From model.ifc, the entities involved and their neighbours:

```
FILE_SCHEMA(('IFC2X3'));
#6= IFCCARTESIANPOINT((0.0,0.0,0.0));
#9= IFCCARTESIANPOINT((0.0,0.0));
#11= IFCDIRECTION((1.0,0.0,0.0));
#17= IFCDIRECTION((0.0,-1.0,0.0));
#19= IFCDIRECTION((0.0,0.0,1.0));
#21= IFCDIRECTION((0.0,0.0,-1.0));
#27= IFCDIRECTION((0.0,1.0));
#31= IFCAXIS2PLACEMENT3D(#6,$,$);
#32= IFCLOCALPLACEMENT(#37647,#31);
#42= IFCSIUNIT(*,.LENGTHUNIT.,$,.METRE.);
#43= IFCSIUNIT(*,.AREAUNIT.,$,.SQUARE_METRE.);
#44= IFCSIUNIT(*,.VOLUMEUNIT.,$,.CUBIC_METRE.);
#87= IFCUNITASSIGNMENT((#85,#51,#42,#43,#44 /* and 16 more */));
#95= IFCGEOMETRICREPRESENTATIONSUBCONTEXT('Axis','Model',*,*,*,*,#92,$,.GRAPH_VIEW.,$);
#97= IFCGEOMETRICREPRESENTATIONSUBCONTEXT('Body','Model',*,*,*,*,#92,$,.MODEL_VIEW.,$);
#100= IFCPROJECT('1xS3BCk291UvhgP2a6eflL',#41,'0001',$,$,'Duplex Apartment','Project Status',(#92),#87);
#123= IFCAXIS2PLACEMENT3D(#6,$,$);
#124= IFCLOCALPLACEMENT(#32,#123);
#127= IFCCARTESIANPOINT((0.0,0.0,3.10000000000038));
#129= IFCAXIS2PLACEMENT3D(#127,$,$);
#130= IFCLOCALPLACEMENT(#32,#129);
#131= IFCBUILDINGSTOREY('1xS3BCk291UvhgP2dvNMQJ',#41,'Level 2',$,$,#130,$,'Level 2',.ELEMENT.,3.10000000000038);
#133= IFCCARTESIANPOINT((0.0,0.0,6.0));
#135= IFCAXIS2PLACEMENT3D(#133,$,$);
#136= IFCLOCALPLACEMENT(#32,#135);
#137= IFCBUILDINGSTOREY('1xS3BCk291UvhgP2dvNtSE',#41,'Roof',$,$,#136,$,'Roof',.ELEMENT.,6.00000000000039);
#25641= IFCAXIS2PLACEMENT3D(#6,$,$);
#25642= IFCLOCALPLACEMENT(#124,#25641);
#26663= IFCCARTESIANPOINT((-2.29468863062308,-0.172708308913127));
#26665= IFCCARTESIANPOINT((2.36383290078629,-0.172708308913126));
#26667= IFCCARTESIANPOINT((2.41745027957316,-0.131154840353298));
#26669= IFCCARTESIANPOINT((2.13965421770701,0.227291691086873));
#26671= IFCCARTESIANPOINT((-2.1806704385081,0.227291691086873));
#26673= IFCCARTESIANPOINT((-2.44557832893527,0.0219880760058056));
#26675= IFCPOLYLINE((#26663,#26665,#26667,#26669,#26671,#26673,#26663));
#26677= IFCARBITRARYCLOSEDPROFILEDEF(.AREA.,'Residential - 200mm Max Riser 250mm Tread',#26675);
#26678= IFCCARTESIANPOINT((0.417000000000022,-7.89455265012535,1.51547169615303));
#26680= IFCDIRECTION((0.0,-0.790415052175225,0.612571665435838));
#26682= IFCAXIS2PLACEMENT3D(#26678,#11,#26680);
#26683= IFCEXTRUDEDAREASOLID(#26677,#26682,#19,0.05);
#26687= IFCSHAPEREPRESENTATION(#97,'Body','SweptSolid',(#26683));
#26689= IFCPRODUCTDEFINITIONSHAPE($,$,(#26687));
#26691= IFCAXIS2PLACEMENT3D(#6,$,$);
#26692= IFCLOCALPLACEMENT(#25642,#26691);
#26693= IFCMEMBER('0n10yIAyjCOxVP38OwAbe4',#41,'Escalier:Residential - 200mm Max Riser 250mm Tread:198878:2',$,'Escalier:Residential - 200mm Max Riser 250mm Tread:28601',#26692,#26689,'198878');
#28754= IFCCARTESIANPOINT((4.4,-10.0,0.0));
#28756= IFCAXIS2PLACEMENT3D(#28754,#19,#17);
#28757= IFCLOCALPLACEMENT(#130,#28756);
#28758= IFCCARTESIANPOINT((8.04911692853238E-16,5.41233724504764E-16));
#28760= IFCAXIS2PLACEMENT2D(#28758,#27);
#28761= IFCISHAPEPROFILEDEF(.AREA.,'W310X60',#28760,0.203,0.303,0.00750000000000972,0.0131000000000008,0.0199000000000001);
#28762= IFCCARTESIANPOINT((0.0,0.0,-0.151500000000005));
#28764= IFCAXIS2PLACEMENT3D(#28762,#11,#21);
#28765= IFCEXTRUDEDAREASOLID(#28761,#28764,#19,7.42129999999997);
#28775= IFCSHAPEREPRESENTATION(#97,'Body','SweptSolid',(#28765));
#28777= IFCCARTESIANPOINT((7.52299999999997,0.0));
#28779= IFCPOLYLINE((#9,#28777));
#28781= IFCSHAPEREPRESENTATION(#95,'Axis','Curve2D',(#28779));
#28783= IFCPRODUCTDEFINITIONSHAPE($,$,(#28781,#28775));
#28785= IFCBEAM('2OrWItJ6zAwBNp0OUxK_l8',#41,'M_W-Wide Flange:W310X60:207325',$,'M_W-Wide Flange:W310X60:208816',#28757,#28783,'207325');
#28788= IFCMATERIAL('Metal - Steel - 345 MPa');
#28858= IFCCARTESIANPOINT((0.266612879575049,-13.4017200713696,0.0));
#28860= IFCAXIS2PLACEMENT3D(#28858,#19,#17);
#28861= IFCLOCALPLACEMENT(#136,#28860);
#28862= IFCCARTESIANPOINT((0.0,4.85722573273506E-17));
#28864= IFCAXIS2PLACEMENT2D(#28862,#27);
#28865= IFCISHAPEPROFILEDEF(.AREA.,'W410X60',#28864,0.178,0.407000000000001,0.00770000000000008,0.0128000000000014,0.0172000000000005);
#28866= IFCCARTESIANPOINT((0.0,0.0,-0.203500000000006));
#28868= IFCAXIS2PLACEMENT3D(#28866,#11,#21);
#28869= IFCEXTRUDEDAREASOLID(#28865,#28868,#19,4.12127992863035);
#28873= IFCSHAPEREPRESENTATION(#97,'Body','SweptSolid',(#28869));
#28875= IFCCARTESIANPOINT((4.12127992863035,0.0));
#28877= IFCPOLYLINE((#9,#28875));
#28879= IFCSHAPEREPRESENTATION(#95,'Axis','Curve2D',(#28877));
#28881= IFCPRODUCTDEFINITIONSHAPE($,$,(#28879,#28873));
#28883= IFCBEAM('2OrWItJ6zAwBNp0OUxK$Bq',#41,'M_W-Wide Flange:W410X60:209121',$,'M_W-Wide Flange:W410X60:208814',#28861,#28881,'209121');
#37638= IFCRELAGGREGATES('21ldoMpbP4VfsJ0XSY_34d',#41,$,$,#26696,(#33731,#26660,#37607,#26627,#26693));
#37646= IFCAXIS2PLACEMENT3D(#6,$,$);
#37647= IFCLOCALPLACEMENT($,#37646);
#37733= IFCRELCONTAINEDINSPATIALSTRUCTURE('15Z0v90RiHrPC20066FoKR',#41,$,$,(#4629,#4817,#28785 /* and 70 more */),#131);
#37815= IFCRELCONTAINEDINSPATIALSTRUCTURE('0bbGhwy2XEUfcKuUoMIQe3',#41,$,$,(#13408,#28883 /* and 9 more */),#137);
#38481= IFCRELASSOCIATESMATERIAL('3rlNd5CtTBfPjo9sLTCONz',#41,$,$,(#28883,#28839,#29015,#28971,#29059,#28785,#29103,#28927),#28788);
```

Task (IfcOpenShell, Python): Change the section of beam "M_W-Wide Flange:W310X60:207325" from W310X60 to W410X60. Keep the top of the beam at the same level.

```python
import ifcopenshell
import ifcopenshell.util.element
import ifcopenshell.util.representation

model = ifcopenshell.open("model.ifc")

member = model.by_guid("2OrWItJ6zAwBNp0OUxK_l8")
source = next(p for p in model.by_type("IfcIShapeProfileDef") if p.ProfileName == "W410X60")

body = ifcopenshell.util.representation.get_representation(member, "Model", "Body")
solid = body.Items[0]
old_profile = solid.SweptArea

# Copy the section's sizes but keep this member's own profile position.
profile = ifcopenshell.util.element.copy(model, source)
# Profiles are centred, so shift by half the change in depth to hold the top.
shift = (old_profile.OverallDepth - profile.OverallDepth) / 2
x, y = old_profile.Position.Location.Coordinates
up = (-1.0, 0.0)  # upwards, in the solid's own plane
location = model.createIfcCartesianPoint((x + up[0] * shift, y + up[1] * shift))
profile.Position = model.createIfcAxis2Placement2D(location, old_profile.Position.RefDirection)
solid.SweptArea = profile
if not model.get_total_inverses(old_profile):
    ifcopenshell.util.element.remove_deep2(model, old_profile)
member.Name = member.Name.replace("W310X60", "W410X60")
member.ObjectType = member.ObjectType.replace("W310X60", "W410X60")

print(solid.SweptArea)

model.write("model_updated.ifc")
```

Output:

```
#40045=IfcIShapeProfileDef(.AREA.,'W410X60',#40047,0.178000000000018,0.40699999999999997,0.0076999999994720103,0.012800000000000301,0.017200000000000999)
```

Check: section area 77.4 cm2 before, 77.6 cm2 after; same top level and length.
